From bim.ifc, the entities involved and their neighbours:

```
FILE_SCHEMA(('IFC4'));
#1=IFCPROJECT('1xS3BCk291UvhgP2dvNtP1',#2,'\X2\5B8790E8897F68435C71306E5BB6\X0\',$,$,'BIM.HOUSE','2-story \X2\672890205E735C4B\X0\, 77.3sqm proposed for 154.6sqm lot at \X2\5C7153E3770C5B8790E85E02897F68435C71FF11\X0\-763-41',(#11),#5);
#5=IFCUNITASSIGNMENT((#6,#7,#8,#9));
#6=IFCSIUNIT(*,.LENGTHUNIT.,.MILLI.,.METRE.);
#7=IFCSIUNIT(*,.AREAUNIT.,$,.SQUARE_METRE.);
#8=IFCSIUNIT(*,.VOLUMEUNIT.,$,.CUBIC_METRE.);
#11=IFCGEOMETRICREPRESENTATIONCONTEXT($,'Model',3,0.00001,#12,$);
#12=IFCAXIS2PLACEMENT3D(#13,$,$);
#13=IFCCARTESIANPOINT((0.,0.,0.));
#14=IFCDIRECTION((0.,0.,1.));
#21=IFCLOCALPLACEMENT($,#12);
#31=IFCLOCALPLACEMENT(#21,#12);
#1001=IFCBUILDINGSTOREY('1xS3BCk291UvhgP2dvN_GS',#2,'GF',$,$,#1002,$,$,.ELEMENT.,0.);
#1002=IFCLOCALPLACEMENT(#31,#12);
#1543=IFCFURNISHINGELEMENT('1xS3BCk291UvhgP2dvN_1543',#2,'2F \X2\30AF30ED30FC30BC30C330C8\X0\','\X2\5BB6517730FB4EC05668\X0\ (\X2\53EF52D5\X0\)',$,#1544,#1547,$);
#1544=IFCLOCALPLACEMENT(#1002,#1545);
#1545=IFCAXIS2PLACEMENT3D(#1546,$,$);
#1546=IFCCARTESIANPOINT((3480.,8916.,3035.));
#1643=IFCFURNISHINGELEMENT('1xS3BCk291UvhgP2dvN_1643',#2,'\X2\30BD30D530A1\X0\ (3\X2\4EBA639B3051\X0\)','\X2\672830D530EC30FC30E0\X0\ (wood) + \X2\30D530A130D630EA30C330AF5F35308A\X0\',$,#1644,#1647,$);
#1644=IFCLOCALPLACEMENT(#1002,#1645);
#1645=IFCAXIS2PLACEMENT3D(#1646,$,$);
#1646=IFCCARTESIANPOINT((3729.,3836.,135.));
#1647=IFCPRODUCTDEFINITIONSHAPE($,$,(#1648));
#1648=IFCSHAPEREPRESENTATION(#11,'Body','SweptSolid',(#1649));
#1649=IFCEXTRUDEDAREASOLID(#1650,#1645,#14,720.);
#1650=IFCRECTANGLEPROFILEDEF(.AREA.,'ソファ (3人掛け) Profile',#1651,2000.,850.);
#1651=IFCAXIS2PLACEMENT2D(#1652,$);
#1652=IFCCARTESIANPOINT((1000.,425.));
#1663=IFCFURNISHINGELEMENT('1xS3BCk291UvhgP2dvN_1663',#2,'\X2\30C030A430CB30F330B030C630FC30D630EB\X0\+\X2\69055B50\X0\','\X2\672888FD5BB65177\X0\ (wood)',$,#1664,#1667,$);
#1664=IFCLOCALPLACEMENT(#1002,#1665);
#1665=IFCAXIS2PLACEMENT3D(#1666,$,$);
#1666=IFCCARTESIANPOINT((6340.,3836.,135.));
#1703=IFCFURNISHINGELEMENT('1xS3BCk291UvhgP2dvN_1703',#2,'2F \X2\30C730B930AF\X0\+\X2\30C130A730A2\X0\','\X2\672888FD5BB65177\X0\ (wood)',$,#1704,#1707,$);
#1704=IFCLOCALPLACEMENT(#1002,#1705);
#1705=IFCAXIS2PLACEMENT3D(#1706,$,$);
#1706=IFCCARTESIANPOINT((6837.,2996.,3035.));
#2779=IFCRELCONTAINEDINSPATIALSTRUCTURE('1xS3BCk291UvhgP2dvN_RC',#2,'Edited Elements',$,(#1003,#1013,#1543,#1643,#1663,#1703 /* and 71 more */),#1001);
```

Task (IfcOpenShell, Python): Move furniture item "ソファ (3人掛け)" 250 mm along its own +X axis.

```python
import ifcopenshell
import ifcopenshell.api.geometry
import ifcopenshell.util.placement
import ifcopenshell.util.unit

model = ifcopenshell.open("bim.ifc")
unit_scale = ifcopenshell.util.unit.calculate_unit_scale(model)

item = model.by_guid("1xS3BCk291UvhgP2dvN_1643")
matrix = ifcopenshell.util.placement.get_local_placement(item.ObjectPlacement)
matrix[:3, 3] += matrix[:3, 0] * 0.25 / unit_scale
ifcopenshell.api.geometry.edit_object_placement(model, product=item, matrix=matrix, is_si=False)

print(ifcopenshell.util.placement.get_local_placement(item.ObjectPlacement).round(3) + 0.0)

model.write("bim-out.ifc")
```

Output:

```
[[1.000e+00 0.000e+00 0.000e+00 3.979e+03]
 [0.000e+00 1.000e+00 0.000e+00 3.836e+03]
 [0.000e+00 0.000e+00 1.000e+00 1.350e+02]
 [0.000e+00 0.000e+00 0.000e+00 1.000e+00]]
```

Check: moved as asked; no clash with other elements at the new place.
